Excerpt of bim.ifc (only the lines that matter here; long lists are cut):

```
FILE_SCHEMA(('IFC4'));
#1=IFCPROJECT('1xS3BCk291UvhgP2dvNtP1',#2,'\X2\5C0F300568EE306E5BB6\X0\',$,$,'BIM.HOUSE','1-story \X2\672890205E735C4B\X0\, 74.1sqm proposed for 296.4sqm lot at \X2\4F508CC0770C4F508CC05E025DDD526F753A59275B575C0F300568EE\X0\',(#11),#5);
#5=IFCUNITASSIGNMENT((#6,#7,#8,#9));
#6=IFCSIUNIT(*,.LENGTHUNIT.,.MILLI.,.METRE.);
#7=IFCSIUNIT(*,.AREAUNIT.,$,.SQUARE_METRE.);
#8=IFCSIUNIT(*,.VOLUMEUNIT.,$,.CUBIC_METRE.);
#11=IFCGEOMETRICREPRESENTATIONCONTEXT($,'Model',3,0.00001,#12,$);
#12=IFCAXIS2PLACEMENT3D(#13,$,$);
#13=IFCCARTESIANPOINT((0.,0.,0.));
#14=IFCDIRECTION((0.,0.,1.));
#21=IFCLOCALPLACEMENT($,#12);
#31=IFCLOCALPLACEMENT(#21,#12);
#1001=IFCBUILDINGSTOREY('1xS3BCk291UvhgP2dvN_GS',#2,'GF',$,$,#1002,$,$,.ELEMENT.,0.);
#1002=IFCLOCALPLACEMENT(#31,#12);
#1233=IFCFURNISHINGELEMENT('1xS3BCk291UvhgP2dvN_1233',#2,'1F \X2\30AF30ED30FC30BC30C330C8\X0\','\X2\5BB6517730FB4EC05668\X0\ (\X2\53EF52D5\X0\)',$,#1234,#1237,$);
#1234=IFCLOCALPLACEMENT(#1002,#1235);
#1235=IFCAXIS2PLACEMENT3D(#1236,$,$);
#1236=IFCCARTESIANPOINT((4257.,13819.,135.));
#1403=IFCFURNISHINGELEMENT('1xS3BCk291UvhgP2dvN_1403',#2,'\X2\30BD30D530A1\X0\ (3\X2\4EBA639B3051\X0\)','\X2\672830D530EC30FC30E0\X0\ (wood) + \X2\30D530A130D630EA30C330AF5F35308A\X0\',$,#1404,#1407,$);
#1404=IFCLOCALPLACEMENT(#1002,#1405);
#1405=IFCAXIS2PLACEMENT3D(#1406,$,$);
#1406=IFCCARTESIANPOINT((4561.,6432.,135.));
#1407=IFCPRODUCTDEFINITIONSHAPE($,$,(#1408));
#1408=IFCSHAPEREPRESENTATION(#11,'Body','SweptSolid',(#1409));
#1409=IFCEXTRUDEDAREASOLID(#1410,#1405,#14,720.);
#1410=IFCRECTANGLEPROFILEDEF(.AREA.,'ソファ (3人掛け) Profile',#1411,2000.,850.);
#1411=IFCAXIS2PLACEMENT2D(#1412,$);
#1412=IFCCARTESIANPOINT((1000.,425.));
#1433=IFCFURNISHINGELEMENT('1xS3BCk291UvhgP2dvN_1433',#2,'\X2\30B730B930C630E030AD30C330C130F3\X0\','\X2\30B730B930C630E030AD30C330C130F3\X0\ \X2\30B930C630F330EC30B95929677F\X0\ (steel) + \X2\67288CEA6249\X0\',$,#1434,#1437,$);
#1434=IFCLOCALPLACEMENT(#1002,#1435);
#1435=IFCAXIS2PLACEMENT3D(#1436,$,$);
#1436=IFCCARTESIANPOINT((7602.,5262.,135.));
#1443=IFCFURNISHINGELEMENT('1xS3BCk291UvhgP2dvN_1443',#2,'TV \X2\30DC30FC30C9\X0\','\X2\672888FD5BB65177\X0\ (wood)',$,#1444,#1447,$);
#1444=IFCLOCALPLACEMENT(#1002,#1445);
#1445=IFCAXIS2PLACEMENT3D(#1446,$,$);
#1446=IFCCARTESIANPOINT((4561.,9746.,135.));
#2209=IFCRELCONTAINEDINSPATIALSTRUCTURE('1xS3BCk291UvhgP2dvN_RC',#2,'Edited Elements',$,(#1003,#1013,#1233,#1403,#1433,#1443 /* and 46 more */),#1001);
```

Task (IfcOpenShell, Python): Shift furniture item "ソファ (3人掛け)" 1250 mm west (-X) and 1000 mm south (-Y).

```python
import ifcopenshell
import ifcopenshell.api.geometry
import ifcopenshell.util.placement
import ifcopenshell.util.unit

model = ifcopenshell.open("bim.ifc")
unit_scale = ifcopenshell.util.unit.calculate_unit_scale(model)

item = model.by_guid("1xS3BCk291UvhgP2dvN_1403")
matrix = ifcopenshell.util.placement.get_local_placement(item.ObjectPlacement)
matrix[0, 3] -= 1.25 / unit_scale
matrix[1, 3] -= 1 / unit_scale
ifcopenshell.api.geometry.edit_object_placement(model, product=item, matrix=matrix, is_si=False)

print(ifcopenshell.util.placement.get_local_placement(item.ObjectPlacement).round(3) + 0.0)

model.write("bim_updated.ifc")
```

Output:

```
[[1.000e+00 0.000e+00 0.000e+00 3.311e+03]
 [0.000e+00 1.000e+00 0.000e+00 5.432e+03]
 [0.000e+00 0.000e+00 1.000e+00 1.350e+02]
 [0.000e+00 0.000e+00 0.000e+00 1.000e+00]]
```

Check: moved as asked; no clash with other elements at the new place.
